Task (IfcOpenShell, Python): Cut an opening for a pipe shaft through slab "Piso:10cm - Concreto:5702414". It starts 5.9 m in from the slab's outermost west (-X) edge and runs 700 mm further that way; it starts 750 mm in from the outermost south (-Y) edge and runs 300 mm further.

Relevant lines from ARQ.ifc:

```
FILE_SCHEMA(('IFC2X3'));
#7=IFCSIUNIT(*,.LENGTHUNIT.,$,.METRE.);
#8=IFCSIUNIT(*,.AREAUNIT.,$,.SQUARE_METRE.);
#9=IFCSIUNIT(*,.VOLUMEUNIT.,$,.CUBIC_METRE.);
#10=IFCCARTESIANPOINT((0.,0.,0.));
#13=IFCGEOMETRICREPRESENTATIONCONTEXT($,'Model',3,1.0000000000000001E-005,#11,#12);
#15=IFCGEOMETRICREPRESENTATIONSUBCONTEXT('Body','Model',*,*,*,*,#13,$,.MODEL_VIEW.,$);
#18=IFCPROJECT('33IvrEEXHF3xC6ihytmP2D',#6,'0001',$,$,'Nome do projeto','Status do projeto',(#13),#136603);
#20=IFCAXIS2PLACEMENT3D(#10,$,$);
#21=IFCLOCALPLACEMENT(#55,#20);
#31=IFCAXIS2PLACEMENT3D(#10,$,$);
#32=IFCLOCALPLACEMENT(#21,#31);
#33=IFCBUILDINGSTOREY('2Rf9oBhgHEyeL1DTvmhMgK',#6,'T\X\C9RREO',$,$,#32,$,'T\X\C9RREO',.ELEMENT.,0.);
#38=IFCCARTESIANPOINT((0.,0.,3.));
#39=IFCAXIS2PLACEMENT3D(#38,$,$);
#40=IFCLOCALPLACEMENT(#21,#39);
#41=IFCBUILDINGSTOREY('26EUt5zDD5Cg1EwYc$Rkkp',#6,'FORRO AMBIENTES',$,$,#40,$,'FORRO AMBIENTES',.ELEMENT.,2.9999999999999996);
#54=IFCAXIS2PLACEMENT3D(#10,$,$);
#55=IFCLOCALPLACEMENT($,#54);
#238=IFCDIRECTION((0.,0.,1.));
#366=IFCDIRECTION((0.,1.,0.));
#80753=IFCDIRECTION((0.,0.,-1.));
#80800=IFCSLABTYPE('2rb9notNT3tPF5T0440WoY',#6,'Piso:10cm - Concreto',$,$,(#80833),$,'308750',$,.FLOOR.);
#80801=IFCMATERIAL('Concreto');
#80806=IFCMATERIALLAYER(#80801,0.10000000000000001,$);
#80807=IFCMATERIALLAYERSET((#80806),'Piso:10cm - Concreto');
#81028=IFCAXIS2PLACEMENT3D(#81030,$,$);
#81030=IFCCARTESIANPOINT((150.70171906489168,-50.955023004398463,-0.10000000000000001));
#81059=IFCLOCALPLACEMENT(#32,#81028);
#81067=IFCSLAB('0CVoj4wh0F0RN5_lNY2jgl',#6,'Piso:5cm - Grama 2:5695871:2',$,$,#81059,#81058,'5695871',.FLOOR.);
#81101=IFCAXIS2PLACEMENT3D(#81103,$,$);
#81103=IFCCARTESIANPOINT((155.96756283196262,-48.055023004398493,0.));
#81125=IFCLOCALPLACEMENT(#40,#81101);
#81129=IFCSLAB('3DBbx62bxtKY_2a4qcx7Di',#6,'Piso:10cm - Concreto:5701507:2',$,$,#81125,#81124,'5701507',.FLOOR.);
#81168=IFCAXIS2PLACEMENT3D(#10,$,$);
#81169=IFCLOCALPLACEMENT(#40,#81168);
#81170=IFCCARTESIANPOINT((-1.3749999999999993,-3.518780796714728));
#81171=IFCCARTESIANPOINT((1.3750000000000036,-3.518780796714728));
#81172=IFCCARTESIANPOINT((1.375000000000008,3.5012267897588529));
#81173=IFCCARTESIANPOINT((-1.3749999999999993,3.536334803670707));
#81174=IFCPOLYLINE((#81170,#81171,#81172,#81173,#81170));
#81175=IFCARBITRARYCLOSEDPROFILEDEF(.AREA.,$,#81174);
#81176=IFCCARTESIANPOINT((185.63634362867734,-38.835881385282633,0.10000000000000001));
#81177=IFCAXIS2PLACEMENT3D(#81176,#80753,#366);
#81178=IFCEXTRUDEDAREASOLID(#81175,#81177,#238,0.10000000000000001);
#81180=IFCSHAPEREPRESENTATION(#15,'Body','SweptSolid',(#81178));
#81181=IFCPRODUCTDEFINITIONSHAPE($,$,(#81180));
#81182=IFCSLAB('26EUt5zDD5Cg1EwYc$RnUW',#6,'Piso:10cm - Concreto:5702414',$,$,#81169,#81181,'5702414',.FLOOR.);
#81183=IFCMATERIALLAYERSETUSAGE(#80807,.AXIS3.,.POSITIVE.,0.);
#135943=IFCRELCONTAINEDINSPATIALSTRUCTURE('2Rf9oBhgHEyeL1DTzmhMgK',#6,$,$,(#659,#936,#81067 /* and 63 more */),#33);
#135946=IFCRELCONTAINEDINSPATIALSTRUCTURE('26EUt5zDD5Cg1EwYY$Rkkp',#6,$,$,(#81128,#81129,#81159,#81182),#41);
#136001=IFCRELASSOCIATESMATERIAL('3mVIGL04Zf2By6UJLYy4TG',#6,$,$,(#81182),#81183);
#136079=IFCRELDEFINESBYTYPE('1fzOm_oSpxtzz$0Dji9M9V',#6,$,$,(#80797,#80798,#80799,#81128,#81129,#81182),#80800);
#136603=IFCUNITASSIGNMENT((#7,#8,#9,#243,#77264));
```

```python
import numpy as np
import ifcopenshell
import ifcopenshell.api.feature
import ifcopenshell.api.geometry
import ifcopenshell.api.root
import ifcopenshell.geom
import ifcopenshell.util.placement
import ifcopenshell.util.representation
import ifcopenshell.util.shape
import ifcopenshell.util.unit

model = ifcopenshell.open("ARQ.ifc")
unit_scale = ifcopenshell.util.unit.calculate_unit_scale(model)
settings = ifcopenshell.geom.settings()


def volume(element):
    """Net volume in cubic metres, openings subtracted."""
    shape = ifcopenshell.geom.create_shape(settings, element)
    return ifcopenshell.util.shape.get_volume(shape.geometry)


slab = model.by_guid("26EUt5zDD5Cg1EwYc$RnUW")
before = volume(slab)

# Extent in the slab's own axes, in metres. The edges named are its -X and -Y sides.
slab_shape = ifcopenshell.geom.create_shape(settings, slab)
vertices = ifcopenshell.util.shape.get_vertices(slab_shape.geometry)
x_min, y_min, bottom = vertices.min(axis=0)
top = vertices[:, 2].max()

opening = ifcopenshell.api.root.create_entity(model, ifc_class="IfcOpeningElement", name="Pipe shaft opening")
context = ifcopenshell.util.representation.get_context(model, "Model", "Body", "MODEL_VIEW")
width, depth = 0.7, 0.3
outline = [(0.0, 0.0), (width, 0.0), (width, depth), (0.0, depth), (0.0, 0.0)]
# Overshoot both faces by 50 mm so the cut is clean.
shape = ifcopenshell.api.geometry.add_slab_representation(
    model, context=context, depth=top - bottom + 0.1, polyline=outline
)
ifcopenshell.api.geometry.assign_representation(model, product=opening, representation=shape)

matrix = ifcopenshell.util.placement.get_local_placement(slab.ObjectPlacement)
matrix[:, 3] = matrix @ np.append(np.array([x_min + 5.9, y_min + 0.75, bottom - 0.05]) / unit_scale, 1.0)
ifcopenshell.api.geometry.edit_object_placement(model, product=opening, matrix=matrix, is_si=False)
ifcopenshell.api.feature.add_feature(model, feature=opening, element=slab)

after = volume(slab)

print(f"slab volume {before:.3f} -> {after:.3f} m3")

model.write("ARQ_updated.ifc")
```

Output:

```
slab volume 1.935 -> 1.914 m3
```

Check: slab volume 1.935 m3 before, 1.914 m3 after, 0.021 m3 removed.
